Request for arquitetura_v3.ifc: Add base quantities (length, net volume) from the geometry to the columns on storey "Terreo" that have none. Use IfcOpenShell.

First a look at what the model holds.

```python
import ifcopenshell
import ifcopenshell.util.element
import ifcopenshell.util.unit

model = ifcopenshell.open("arquitetura_v3.ifc")
print(model.schema)
for unit_type in ("LENGTHUNIT", "AREAUNIT", "VOLUMEUNIT"):
    print(unit_type, ifcopenshell.util.unit.calculate_unit_scale(model, unit_type))
storey = next(s for s in model.by_type("IfcBuildingStorey") if s.Name == "Terreo")
columns = [e for e in ifcopenshell.util.element.get_decomposition(storey) if e.is_a("IfcColumn")]
for e in sorted(columns, key=lambda e: e.id()):
    print(e.id(), e.is_a(), e.Name, list(ifcopenshell.util.element.get_psets(e, qtos_only=True)), sep=" | ")
```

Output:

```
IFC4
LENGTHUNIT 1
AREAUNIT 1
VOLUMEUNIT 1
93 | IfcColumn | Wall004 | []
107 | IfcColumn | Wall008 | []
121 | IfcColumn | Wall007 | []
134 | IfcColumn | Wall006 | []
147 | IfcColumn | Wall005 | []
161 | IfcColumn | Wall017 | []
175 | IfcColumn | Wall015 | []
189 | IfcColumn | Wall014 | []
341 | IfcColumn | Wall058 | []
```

```python
import ifcopenshell
import ifcopenshell.api.pset
import ifcopenshell.geom
import ifcopenshell.util.element
import ifcopenshell.util.shape
import ifcopenshell.util.unit

model = ifcopenshell.open("arquitetura_v3.ifc")
unit_scale = ifcopenshell.util.unit.calculate_unit_scale(model)
volume_scale = ifcopenshell.util.unit.calculate_unit_scale(model, "VOLUMEUNIT")
settings = ifcopenshell.geom.settings()

storey = next(s for s in model.by_type("IfcBuildingStorey") if s.Name == "Terreo")
columns = [e for e in ifcopenshell.util.element.get_decomposition(storey) if e.is_a("IfcColumn")]

for e in sorted(columns, key=lambda e: e.id()):
    if ifcopenshell.util.element.get_psets(e, qtos_only=True, should_inherit=False):
        continue
    # Geometry comes back in metres, in the element's own axes.
    shape = ifcopenshell.geom.create_shape(settings, e)
    values = {
        "Length": ifcopenshell.util.shape.get_z(shape.geometry) / unit_scale,
        "NetVolume": ifcopenshell.util.shape.get_volume(shape.geometry) / volume_scale,
    }
    qto = ifcopenshell.api.pset.add_qto(model, product=e, name="Qto_ColumnBaseQuantities")
    ifcopenshell.api.pset.edit_qto(model, qto=qto, properties=values)
    print(e.id(), {k: round(v, 3) for k, v in values.items()})

model.write("arquitetura_v3_rev.ifc")
```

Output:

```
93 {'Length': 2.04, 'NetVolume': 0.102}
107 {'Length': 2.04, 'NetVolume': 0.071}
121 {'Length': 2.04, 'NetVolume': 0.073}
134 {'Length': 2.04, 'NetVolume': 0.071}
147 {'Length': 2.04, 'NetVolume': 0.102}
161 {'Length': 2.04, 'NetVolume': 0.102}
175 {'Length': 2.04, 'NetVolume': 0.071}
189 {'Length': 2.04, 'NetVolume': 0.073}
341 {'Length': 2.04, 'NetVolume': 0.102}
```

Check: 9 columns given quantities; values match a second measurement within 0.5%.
